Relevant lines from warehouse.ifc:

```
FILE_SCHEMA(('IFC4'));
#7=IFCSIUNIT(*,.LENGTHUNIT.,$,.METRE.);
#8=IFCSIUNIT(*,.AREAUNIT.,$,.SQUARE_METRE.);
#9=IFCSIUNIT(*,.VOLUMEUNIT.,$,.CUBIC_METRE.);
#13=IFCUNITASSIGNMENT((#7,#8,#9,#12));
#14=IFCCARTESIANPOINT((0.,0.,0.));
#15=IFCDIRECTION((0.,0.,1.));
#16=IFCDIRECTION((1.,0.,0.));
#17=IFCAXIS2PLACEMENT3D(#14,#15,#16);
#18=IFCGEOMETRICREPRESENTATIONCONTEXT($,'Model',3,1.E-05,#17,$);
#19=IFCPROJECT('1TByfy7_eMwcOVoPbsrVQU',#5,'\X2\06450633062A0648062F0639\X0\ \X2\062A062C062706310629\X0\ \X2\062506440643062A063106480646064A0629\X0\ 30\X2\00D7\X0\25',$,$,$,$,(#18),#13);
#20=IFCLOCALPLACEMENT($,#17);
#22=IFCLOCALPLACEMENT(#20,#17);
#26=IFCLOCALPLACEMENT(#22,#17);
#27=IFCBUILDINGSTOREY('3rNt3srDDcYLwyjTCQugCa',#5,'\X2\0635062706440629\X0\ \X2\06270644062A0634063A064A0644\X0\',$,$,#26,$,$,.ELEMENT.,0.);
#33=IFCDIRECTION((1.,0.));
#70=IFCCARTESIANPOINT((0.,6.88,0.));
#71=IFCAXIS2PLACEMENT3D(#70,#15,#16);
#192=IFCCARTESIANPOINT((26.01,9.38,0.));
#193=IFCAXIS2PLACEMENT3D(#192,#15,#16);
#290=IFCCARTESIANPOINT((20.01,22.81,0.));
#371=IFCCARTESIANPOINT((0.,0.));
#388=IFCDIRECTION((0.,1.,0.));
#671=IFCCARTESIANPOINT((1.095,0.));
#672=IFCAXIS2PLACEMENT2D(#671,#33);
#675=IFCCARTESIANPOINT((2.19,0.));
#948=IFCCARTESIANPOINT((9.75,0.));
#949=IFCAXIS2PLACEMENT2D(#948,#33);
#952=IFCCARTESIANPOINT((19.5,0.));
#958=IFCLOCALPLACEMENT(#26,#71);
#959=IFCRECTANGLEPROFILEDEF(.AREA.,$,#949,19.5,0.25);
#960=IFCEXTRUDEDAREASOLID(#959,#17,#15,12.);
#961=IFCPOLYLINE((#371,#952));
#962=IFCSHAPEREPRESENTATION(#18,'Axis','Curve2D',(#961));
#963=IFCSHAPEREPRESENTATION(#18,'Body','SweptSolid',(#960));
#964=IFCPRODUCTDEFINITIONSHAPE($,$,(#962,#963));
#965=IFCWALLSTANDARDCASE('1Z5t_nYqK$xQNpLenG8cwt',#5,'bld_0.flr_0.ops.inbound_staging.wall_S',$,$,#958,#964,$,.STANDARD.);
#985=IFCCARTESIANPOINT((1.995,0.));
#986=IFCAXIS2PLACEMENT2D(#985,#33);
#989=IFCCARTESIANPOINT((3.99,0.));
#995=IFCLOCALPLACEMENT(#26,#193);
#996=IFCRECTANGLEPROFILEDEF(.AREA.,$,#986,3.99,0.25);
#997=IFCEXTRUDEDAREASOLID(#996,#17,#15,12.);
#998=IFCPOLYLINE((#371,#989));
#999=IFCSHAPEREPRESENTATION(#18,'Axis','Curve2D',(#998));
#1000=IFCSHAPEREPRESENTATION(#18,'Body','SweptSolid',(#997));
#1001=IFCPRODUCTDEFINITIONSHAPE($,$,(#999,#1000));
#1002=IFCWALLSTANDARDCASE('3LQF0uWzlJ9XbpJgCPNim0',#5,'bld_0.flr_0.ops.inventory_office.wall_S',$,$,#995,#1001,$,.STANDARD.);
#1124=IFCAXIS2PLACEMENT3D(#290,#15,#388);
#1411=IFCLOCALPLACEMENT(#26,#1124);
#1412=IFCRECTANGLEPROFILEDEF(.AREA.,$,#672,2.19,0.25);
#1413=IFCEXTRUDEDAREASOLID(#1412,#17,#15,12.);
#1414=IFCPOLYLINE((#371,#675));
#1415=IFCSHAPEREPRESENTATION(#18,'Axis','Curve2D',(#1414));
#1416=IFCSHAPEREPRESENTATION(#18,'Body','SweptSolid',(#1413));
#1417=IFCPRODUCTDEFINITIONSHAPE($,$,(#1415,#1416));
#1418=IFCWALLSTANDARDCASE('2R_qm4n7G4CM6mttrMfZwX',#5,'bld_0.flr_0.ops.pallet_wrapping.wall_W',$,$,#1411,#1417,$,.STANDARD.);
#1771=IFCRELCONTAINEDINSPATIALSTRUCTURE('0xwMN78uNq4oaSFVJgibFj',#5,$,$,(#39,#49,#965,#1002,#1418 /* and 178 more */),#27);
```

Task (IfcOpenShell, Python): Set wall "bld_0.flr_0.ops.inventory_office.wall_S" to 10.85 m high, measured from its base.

```python
import ifcopenshell
import ifcopenshell.geom
import ifcopenshell.util.shape

model = ifcopenshell.open("warehouse.ifc")
settings = ifcopenshell.geom.settings()


def volume(element):
    """Net volume in cubic metres, openings subtracted."""
    shape = ifcopenshell.geom.create_shape(settings, element)
    return ifcopenshell.util.shape.get_volume(shape.geometry)


wall = model.by_id(1002)
before = volume(wall)

body = next(r for r in wall.Representation.Representations if r.RepresentationIdentifier == "Body")
solid = body.Items[0]
old_height = solid.Depth
solid.Depth = 10.85
after = volume(wall)

print(f"height {old_height:g} -> {solid.Depth:g}, volume {before:.3f} -> {after:.3f} m3")

model.write("warehouse_updated.ifc")
```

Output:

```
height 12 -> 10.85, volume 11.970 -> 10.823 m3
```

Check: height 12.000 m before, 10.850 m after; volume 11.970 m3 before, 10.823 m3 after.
